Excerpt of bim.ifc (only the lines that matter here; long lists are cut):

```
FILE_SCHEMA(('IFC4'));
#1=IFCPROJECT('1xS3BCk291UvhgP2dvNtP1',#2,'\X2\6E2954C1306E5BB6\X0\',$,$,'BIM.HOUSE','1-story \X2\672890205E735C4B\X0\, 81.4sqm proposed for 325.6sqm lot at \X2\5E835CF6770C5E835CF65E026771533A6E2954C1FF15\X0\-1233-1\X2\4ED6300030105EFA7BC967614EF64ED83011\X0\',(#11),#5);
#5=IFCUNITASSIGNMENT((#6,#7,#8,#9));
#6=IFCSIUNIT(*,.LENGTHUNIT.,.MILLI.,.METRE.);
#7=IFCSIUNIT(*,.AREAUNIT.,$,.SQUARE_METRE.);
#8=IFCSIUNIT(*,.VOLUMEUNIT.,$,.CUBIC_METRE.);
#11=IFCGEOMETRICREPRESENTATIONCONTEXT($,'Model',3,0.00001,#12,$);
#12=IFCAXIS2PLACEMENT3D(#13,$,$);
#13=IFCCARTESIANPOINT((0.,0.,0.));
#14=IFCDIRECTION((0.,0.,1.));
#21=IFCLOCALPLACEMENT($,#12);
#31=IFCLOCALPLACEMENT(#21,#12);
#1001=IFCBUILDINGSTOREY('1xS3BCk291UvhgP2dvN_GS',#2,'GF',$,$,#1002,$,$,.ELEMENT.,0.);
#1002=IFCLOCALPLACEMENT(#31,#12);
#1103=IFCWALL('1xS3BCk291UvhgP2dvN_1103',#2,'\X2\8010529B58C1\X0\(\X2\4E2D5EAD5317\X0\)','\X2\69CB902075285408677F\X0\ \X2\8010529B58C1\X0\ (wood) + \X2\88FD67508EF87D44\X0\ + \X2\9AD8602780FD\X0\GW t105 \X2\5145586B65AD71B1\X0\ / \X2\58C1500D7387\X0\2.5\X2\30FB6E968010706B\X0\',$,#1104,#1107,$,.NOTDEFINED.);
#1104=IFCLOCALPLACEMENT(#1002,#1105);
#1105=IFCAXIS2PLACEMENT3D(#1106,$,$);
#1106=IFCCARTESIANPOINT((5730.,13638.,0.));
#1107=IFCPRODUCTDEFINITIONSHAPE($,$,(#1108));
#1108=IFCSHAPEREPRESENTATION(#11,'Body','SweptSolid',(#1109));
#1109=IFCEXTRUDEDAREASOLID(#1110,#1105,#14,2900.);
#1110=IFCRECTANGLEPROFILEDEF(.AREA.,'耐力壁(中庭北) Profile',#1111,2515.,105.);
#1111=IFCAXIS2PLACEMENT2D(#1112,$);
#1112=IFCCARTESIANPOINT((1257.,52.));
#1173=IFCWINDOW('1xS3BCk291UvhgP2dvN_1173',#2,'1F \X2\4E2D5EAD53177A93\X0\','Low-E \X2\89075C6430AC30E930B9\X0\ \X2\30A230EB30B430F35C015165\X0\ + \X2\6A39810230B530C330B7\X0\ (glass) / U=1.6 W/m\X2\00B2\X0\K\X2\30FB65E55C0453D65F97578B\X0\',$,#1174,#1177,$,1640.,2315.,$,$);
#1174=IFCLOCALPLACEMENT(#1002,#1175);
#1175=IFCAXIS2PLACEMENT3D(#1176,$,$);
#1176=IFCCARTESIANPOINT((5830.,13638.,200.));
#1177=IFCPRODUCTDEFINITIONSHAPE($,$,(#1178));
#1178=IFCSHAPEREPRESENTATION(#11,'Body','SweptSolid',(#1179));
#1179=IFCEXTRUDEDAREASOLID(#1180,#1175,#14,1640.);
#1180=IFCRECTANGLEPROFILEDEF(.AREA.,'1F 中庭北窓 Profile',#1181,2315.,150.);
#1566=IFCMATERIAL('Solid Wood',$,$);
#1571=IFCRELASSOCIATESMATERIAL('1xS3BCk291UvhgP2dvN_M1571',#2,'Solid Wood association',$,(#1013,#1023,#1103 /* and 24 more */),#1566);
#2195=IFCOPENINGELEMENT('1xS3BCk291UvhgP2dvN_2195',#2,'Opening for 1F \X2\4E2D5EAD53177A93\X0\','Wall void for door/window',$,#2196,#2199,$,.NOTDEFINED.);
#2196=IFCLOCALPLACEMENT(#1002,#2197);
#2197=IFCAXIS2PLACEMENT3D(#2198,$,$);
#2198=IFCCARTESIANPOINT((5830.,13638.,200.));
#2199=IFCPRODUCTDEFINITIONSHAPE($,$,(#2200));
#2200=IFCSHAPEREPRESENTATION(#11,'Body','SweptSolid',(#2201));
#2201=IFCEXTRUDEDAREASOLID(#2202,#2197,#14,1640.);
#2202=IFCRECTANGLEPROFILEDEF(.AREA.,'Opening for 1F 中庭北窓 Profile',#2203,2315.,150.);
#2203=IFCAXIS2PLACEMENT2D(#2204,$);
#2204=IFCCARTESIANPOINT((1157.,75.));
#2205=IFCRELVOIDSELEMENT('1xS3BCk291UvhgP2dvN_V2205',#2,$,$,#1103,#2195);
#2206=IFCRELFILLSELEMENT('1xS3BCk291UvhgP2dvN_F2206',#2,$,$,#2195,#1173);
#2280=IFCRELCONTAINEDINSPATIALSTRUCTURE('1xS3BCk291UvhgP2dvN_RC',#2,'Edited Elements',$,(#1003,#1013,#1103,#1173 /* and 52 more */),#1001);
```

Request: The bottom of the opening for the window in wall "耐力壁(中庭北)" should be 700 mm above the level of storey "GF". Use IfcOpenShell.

```python
import numpy as np
import ifcopenshell
import ifcopenshell.api.geometry
import ifcopenshell.geom
import ifcopenshell.util.element
import ifcopenshell.util.placement
import ifcopenshell.util.shape
import ifcopenshell.util.unit

model = ifcopenshell.open("bim.ifc")
unit_scale = ifcopenshell.util.unit.calculate_unit_scale(model)

window = model.by_id(1173)
opening = window.FillsVoids[0].RelatingOpeningElement
storey = ifcopenshell.util.element.get_container(window, ifc_class="IfcBuildingStorey")
level = ifcopenshell.util.placement.get_local_placement(storey.ObjectPlacement)[2, 3]

# The opening's origin need not be at the sill, so measure its lowest point.
shape = ifcopenshell.geom.create_shape(ifcopenshell.geom.settings(), opening)
bottom = ifcopenshell.util.shape.get_shape_bottom_elevation(shape, shape.geometry) / unit_scale
dz = level + 0.7 / unit_scale - bottom

shift = np.array([0.0, 0.0, dz])
# The window is not placed relative to its opening, so move both.
for product in (opening, window):
    matrix = ifcopenshell.util.placement.get_local_placement(product.ObjectPlacement)
    matrix[:3, 3] += shift
    ifcopenshell.api.geometry.edit_object_placement(model, product=product, matrix=matrix, is_si=False)

print(f"moved by {dz * unit_scale:+.3f} m")

model.write("bim_updated.ifc")
```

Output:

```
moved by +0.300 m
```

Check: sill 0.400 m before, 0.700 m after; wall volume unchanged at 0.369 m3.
